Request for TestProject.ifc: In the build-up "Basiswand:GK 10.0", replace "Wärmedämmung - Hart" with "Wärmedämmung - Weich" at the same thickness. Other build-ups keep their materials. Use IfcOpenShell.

First a look at what the model holds.

```python
import ifcopenshell
import ifcopenshell.util.element

model = ifcopenshell.open("TestProject.ifc")
print(model.schema)
for layer_set in model.by_type("IfcMaterialLayerSet"):
    if layer_set.LayerSetName == "Basiswand:GK 10.0":
        for layer in layer_set.MaterialLayers:
            print(layer.id(), layer.Material and layer.Material.Name, layer.LayerThickness, sep=" | ")
        print(len(ifcopenshell.util.element.get_elements_by_material(model, layer_set)), "elements and types use it")
print(sorted(m.Name for m in model.by_type("IfcMaterial") if m.Name)[:60])
```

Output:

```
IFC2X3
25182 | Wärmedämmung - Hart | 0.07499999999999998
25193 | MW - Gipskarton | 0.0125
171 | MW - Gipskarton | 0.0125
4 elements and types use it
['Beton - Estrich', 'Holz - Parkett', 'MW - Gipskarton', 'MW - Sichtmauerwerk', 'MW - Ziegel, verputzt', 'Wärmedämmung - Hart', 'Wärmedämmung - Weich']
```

```python
import ifcopenshell
import ifcopenshell.api.material

model = ifcopenshell.open("TestProject.ifc")

layer_set = next(s for s in model.by_type("IfcMaterialLayerSet") if s.LayerSetName == "Basiswand:GK 10.0")
layer = next(l for l in layer_set.MaterialLayers if l.Material and l.Material.Name == "Wärmedämmung - Hart")
material = next(m for m in model.by_type("IfcMaterial") if m.Name == "Wärmedämmung - Weich")

# Point this one layer at the other material; renaming the old one would change it everywhere.
ifcopenshell.api.material.edit_layer(model, layer=layer, attributes={}, material=material)

print([l.Material.Name if l.Material else None for l in layer_set.MaterialLayers])

model.write("TestProject_updated.ifc")
```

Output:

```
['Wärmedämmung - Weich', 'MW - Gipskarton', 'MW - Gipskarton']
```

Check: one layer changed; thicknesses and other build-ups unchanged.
